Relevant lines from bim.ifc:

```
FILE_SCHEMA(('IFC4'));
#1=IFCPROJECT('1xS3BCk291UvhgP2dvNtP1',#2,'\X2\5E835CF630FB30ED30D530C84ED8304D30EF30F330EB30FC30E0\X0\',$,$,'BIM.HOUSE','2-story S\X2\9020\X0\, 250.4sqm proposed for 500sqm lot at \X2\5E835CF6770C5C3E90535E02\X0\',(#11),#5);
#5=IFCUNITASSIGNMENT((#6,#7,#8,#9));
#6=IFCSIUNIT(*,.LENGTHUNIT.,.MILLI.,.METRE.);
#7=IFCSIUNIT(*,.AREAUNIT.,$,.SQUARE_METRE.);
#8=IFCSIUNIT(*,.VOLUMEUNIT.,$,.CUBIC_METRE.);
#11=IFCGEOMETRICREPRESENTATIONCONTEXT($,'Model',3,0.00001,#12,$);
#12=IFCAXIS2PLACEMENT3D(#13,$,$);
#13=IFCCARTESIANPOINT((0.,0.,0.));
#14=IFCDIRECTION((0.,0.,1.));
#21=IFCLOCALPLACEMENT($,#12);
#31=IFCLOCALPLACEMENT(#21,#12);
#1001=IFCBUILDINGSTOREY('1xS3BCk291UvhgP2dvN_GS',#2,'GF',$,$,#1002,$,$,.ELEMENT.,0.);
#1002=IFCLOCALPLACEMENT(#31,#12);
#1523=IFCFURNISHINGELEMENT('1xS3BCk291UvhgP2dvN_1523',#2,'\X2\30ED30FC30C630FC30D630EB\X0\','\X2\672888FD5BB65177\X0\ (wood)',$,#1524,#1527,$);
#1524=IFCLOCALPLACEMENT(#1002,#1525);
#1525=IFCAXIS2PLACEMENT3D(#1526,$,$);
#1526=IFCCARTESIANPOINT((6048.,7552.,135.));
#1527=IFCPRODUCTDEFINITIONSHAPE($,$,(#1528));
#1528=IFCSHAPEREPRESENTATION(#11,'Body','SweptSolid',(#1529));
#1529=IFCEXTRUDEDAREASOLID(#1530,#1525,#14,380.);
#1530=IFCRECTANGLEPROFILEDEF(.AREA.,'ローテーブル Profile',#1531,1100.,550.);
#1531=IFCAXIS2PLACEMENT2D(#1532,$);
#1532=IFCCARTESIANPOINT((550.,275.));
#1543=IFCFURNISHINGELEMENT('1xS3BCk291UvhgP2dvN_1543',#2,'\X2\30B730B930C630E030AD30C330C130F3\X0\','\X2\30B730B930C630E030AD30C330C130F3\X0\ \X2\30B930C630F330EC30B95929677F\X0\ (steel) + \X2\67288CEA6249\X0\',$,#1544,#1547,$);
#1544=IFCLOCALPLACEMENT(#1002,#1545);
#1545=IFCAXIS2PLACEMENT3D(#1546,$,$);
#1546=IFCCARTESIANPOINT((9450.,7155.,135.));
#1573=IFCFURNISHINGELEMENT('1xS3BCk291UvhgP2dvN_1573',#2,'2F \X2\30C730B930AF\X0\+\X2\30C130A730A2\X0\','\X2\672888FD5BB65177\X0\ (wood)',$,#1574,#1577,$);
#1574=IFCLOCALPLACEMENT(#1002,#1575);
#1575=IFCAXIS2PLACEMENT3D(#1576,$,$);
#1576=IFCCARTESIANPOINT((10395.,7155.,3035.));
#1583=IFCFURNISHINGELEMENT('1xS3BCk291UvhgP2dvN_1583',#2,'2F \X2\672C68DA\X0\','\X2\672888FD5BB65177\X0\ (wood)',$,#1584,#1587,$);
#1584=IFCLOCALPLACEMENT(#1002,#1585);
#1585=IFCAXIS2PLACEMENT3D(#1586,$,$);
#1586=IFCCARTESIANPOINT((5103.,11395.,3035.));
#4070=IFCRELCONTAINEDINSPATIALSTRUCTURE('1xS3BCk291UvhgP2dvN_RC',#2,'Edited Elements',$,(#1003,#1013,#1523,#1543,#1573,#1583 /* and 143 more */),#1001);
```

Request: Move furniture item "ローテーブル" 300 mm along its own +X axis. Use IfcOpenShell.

```python
import ifcopenshell
import ifcopenshell.api.geometry
import ifcopenshell.util.placement

model = ifcopenshell.open("bim.ifc")

item = model.by_id(1523)
matrix = ifcopenshell.util.placement.get_local_placement(item.ObjectPlacement)
matrix[:3, 3] += matrix[:3, 0] * 300.0
ifcopenshell.api.geometry.edit_object_placement(model, product=item, matrix=matrix, is_si=False)

print(ifcopenshell.util.placement.get_local_placement(item.ObjectPlacement).round(3) + 0.0)

model.write("bim_updated.ifc")
```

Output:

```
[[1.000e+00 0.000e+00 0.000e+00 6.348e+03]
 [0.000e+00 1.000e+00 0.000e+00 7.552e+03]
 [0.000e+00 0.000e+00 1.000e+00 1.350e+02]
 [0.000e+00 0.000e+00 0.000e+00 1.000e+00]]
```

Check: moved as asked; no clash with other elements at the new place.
